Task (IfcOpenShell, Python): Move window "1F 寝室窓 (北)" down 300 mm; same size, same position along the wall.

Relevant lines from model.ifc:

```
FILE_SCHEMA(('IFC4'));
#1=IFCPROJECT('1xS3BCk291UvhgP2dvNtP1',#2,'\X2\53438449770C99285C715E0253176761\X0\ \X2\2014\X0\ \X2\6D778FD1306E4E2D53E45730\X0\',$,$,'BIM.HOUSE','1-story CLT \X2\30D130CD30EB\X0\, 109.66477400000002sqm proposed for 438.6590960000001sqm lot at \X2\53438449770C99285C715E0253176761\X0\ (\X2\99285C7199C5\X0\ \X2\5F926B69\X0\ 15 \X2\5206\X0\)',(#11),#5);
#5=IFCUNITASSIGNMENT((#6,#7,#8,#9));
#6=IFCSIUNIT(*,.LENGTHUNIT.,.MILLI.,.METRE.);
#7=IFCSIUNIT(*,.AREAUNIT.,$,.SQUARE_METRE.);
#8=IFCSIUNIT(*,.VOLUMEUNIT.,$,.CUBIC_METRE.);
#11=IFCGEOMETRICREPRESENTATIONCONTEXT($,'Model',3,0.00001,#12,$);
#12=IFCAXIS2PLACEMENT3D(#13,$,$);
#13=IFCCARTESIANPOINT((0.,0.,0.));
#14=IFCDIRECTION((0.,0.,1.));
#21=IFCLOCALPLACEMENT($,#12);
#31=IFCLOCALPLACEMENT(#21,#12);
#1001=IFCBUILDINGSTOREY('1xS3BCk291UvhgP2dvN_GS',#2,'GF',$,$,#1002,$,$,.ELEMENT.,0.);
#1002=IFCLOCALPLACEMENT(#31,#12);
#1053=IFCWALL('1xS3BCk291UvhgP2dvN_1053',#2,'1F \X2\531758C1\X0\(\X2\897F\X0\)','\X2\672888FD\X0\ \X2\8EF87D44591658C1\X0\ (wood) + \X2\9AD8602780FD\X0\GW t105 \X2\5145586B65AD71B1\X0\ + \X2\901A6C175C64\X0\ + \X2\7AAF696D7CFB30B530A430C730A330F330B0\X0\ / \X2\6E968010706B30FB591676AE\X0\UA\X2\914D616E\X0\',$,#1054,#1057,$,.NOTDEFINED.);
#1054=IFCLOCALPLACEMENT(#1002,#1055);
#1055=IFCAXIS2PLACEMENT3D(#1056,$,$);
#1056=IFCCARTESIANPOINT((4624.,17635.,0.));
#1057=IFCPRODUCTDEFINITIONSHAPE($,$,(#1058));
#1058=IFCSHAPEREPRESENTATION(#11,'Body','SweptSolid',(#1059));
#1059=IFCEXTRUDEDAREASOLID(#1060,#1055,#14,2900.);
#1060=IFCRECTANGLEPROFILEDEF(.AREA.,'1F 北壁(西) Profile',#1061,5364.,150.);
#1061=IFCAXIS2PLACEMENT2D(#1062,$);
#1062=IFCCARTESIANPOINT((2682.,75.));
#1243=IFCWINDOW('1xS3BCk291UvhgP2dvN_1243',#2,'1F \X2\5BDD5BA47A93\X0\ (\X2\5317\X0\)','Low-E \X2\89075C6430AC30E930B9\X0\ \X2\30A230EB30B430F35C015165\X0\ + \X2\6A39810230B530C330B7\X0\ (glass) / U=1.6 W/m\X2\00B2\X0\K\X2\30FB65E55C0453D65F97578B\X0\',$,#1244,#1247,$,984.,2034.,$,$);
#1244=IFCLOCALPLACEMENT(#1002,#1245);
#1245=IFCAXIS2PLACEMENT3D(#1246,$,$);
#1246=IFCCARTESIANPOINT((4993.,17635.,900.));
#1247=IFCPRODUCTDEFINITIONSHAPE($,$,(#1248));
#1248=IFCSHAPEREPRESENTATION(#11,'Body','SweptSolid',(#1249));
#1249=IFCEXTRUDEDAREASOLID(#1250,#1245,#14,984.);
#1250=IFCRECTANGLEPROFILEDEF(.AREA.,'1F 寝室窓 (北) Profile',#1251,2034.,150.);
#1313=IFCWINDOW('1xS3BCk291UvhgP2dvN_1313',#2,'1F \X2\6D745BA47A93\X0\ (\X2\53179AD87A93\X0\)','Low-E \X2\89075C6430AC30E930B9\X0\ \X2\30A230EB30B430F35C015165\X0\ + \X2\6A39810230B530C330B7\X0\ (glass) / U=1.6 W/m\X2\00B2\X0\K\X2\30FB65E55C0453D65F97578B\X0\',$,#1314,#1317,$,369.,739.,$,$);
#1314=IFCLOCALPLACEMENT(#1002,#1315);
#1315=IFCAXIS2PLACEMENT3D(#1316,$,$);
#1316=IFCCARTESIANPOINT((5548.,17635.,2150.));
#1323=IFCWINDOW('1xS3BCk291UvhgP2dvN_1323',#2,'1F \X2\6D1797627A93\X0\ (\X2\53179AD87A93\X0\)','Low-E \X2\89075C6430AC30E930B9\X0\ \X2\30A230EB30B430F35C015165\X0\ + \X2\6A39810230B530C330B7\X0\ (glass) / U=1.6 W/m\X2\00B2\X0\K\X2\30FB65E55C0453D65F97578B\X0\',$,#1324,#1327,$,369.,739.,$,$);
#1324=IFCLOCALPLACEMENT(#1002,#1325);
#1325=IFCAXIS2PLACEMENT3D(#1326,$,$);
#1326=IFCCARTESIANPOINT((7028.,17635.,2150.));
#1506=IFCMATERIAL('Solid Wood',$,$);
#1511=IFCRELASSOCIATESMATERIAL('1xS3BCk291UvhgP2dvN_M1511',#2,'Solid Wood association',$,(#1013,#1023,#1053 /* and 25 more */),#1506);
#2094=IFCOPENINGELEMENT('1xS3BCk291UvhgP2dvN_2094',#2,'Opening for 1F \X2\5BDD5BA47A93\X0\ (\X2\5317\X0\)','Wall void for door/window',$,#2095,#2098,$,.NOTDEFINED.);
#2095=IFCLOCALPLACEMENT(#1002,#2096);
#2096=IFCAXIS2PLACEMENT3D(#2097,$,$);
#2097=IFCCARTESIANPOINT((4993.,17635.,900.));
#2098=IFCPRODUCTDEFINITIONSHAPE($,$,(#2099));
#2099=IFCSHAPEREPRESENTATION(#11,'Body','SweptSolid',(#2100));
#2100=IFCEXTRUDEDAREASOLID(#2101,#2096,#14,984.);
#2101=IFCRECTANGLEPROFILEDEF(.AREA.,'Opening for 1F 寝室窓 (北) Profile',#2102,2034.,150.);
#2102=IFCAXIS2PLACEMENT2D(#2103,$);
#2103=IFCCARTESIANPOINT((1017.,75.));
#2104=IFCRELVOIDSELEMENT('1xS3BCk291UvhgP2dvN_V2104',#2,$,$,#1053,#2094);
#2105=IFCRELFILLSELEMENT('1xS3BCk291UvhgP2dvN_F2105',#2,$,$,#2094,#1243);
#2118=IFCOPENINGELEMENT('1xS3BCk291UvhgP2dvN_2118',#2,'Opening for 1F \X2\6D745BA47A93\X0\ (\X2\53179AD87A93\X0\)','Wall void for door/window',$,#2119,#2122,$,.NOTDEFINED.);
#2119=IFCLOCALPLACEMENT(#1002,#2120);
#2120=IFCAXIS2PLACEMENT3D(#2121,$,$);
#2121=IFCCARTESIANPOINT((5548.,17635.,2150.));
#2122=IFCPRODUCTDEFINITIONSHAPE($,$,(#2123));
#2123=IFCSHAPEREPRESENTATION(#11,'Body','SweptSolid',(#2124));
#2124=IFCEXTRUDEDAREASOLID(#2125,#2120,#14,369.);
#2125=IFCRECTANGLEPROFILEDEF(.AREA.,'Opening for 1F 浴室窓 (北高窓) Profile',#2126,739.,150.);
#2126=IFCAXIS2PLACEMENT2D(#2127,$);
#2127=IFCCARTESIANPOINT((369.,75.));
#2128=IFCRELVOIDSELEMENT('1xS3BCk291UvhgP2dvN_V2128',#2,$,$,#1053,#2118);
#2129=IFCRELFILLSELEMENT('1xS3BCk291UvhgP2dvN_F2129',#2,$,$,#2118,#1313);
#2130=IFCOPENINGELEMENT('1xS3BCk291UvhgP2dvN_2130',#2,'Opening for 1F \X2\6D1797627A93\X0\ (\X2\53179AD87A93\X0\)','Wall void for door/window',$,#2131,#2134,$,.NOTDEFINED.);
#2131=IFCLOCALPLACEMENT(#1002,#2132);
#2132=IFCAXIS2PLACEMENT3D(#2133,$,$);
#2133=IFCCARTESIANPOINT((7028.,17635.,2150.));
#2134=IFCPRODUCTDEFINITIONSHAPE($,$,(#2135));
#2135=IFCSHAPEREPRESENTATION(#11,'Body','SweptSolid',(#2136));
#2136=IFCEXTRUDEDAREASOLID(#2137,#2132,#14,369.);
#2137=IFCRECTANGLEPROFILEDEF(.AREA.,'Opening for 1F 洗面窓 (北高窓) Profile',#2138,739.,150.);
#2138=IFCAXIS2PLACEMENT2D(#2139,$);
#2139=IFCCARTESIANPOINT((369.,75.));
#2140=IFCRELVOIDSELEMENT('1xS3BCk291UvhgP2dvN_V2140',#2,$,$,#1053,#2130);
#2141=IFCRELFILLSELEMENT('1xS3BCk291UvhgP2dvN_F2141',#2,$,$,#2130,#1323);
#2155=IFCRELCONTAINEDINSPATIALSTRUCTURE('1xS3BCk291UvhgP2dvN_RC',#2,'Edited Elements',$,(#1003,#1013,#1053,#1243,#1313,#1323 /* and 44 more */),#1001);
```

```python
import numpy as np
import ifcopenshell
import ifcopenshell.api.geometry
import ifcopenshell.util.placement
import ifcopenshell.util.unit

model = ifcopenshell.open("model.ifc")
unit_scale = ifcopenshell.util.unit.calculate_unit_scale(model)

window = model.by_guid("1xS3BCk291UvhgP2dvN_1243")
opening = window.FillsVoids[0].RelatingOpeningElement
dz = -0.3 / unit_scale

shift = np.array([0.0, 0.0, dz])
# The window is not placed relative to its opening, so move both.
for product in (opening, window):
    matrix = ifcopenshell.util.placement.get_local_placement(product.ObjectPlacement)
    matrix[:3, 3] += shift
    ifcopenshell.api.geometry.edit_object_placement(model, product=product, matrix=matrix, is_si=False)

print(f"moved by {dz * unit_scale:+.3f} m")

model.write("model_v2.ifc")
```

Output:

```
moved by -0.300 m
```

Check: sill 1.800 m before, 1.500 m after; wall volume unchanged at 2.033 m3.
